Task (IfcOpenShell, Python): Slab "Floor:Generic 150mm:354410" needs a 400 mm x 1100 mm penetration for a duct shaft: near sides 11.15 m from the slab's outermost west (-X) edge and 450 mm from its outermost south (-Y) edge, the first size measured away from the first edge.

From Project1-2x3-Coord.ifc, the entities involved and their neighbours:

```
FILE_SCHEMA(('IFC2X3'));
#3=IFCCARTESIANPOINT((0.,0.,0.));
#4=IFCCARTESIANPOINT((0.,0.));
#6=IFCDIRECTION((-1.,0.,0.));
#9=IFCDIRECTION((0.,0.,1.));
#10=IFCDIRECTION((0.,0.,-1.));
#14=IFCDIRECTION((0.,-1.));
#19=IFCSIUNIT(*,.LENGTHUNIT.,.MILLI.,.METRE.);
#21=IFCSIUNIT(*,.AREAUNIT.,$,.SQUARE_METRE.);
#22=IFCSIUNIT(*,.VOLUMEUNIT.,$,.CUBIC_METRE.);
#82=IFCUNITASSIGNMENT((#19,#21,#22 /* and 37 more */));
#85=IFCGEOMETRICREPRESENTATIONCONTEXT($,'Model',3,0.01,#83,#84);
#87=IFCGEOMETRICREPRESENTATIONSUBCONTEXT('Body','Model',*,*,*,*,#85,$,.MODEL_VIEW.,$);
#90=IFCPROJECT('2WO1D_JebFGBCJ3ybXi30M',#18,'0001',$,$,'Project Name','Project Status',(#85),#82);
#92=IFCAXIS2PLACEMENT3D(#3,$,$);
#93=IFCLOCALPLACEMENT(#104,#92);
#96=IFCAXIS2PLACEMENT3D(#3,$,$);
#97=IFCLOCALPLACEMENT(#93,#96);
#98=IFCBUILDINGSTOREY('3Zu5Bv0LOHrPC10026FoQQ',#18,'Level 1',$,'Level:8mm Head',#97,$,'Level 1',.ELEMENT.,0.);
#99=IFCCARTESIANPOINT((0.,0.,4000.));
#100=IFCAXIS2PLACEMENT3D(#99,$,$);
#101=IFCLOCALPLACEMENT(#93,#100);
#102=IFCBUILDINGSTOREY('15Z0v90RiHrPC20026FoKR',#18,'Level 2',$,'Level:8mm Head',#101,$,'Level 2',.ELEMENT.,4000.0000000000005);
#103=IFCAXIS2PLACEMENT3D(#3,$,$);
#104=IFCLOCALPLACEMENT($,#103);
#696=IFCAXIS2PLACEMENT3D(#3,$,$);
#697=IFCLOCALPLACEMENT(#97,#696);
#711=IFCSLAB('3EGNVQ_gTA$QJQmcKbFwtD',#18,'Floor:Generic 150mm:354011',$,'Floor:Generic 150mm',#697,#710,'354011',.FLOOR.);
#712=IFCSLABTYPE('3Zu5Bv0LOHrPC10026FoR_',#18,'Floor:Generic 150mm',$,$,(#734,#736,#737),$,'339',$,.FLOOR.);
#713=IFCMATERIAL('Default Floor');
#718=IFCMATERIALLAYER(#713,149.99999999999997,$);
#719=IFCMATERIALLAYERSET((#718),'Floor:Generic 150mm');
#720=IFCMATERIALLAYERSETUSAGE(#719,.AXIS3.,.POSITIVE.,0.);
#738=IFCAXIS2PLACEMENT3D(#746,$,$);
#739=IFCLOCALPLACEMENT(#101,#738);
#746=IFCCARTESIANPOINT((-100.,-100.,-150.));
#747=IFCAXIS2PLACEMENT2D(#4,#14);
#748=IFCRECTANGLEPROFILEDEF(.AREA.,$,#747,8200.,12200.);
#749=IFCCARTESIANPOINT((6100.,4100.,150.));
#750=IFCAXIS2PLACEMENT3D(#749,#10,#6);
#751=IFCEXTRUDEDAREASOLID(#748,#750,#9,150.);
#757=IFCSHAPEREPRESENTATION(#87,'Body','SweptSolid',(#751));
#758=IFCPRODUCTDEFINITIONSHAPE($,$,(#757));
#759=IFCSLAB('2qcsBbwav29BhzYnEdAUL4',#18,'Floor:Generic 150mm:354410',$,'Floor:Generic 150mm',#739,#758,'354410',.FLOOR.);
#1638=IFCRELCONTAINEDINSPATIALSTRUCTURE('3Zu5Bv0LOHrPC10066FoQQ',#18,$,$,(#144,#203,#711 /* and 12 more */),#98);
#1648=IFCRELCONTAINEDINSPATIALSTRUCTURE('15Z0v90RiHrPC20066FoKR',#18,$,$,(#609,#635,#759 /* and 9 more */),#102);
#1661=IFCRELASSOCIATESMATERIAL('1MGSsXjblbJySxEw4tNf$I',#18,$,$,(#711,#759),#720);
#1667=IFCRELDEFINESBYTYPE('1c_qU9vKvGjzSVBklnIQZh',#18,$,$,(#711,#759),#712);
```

```python
import numpy as np
import ifcopenshell
import ifcopenshell.api.feature
import ifcopenshell.api.geometry
import ifcopenshell.api.root
import ifcopenshell.geom
import ifcopenshell.util.placement
import ifcopenshell.util.representation
import ifcopenshell.util.shape
import ifcopenshell.util.unit

model = ifcopenshell.open("Project1-2x3-Coord.ifc")
unit_scale = ifcopenshell.util.unit.calculate_unit_scale(model)
settings = ifcopenshell.geom.settings()


def volume(element):
    """Net volume in cubic metres, openings subtracted."""
    shape = ifcopenshell.geom.create_shape(settings, element)
    return ifcopenshell.util.shape.get_volume(shape.geometry)


slab = model.by_id(759)
before = volume(slab)

# Extent in the slab's own axes, in metres. The edges named are its -X and -Y sides.
slab_shape = ifcopenshell.geom.create_shape(settings, slab)
vertices = ifcopenshell.util.shape.get_vertices(slab_shape.geometry)
x_min, y_min, bottom = vertices.min(axis=0)
top = vertices[:, 2].max()

opening = ifcopenshell.api.root.create_entity(model, ifc_class="IfcOpeningElement", name="Duct shaft opening")
context = ifcopenshell.util.representation.get_context(model, "Model", "Body", "MODEL_VIEW")
width, depth = 0.4, 1.1
outline = [(0.0, 0.0), (width, 0.0), (width, depth), (0.0, depth), (0.0, 0.0)]
# Overshoot both faces by 50 mm so the cut is clean.
shape = ifcopenshell.api.geometry.add_slab_representation(
    model, context=context, depth=top - bottom + 0.1, polyline=outline
)
ifcopenshell.api.geometry.assign_representation(model, product=opening, representation=shape)

matrix = ifcopenshell.util.placement.get_local_placement(slab.ObjectPlacement)
matrix[:, 3] = matrix @ np.append(np.array([x_min + 11.15, y_min + 0.45, bottom - 0.05]) / unit_scale, 1.0)
ifcopenshell.api.geometry.edit_object_placement(model, product=opening, matrix=matrix, is_si=False)
ifcopenshell.api.feature.add_feature(model, feature=opening, element=slab)

after = volume(slab)

print(f"slab volume {before:.3f} -> {after:.3f} m3")

model.write("Project1-2x3-Coord_v2.ifc")
```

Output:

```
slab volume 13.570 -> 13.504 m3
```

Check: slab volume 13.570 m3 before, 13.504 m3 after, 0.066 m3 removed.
